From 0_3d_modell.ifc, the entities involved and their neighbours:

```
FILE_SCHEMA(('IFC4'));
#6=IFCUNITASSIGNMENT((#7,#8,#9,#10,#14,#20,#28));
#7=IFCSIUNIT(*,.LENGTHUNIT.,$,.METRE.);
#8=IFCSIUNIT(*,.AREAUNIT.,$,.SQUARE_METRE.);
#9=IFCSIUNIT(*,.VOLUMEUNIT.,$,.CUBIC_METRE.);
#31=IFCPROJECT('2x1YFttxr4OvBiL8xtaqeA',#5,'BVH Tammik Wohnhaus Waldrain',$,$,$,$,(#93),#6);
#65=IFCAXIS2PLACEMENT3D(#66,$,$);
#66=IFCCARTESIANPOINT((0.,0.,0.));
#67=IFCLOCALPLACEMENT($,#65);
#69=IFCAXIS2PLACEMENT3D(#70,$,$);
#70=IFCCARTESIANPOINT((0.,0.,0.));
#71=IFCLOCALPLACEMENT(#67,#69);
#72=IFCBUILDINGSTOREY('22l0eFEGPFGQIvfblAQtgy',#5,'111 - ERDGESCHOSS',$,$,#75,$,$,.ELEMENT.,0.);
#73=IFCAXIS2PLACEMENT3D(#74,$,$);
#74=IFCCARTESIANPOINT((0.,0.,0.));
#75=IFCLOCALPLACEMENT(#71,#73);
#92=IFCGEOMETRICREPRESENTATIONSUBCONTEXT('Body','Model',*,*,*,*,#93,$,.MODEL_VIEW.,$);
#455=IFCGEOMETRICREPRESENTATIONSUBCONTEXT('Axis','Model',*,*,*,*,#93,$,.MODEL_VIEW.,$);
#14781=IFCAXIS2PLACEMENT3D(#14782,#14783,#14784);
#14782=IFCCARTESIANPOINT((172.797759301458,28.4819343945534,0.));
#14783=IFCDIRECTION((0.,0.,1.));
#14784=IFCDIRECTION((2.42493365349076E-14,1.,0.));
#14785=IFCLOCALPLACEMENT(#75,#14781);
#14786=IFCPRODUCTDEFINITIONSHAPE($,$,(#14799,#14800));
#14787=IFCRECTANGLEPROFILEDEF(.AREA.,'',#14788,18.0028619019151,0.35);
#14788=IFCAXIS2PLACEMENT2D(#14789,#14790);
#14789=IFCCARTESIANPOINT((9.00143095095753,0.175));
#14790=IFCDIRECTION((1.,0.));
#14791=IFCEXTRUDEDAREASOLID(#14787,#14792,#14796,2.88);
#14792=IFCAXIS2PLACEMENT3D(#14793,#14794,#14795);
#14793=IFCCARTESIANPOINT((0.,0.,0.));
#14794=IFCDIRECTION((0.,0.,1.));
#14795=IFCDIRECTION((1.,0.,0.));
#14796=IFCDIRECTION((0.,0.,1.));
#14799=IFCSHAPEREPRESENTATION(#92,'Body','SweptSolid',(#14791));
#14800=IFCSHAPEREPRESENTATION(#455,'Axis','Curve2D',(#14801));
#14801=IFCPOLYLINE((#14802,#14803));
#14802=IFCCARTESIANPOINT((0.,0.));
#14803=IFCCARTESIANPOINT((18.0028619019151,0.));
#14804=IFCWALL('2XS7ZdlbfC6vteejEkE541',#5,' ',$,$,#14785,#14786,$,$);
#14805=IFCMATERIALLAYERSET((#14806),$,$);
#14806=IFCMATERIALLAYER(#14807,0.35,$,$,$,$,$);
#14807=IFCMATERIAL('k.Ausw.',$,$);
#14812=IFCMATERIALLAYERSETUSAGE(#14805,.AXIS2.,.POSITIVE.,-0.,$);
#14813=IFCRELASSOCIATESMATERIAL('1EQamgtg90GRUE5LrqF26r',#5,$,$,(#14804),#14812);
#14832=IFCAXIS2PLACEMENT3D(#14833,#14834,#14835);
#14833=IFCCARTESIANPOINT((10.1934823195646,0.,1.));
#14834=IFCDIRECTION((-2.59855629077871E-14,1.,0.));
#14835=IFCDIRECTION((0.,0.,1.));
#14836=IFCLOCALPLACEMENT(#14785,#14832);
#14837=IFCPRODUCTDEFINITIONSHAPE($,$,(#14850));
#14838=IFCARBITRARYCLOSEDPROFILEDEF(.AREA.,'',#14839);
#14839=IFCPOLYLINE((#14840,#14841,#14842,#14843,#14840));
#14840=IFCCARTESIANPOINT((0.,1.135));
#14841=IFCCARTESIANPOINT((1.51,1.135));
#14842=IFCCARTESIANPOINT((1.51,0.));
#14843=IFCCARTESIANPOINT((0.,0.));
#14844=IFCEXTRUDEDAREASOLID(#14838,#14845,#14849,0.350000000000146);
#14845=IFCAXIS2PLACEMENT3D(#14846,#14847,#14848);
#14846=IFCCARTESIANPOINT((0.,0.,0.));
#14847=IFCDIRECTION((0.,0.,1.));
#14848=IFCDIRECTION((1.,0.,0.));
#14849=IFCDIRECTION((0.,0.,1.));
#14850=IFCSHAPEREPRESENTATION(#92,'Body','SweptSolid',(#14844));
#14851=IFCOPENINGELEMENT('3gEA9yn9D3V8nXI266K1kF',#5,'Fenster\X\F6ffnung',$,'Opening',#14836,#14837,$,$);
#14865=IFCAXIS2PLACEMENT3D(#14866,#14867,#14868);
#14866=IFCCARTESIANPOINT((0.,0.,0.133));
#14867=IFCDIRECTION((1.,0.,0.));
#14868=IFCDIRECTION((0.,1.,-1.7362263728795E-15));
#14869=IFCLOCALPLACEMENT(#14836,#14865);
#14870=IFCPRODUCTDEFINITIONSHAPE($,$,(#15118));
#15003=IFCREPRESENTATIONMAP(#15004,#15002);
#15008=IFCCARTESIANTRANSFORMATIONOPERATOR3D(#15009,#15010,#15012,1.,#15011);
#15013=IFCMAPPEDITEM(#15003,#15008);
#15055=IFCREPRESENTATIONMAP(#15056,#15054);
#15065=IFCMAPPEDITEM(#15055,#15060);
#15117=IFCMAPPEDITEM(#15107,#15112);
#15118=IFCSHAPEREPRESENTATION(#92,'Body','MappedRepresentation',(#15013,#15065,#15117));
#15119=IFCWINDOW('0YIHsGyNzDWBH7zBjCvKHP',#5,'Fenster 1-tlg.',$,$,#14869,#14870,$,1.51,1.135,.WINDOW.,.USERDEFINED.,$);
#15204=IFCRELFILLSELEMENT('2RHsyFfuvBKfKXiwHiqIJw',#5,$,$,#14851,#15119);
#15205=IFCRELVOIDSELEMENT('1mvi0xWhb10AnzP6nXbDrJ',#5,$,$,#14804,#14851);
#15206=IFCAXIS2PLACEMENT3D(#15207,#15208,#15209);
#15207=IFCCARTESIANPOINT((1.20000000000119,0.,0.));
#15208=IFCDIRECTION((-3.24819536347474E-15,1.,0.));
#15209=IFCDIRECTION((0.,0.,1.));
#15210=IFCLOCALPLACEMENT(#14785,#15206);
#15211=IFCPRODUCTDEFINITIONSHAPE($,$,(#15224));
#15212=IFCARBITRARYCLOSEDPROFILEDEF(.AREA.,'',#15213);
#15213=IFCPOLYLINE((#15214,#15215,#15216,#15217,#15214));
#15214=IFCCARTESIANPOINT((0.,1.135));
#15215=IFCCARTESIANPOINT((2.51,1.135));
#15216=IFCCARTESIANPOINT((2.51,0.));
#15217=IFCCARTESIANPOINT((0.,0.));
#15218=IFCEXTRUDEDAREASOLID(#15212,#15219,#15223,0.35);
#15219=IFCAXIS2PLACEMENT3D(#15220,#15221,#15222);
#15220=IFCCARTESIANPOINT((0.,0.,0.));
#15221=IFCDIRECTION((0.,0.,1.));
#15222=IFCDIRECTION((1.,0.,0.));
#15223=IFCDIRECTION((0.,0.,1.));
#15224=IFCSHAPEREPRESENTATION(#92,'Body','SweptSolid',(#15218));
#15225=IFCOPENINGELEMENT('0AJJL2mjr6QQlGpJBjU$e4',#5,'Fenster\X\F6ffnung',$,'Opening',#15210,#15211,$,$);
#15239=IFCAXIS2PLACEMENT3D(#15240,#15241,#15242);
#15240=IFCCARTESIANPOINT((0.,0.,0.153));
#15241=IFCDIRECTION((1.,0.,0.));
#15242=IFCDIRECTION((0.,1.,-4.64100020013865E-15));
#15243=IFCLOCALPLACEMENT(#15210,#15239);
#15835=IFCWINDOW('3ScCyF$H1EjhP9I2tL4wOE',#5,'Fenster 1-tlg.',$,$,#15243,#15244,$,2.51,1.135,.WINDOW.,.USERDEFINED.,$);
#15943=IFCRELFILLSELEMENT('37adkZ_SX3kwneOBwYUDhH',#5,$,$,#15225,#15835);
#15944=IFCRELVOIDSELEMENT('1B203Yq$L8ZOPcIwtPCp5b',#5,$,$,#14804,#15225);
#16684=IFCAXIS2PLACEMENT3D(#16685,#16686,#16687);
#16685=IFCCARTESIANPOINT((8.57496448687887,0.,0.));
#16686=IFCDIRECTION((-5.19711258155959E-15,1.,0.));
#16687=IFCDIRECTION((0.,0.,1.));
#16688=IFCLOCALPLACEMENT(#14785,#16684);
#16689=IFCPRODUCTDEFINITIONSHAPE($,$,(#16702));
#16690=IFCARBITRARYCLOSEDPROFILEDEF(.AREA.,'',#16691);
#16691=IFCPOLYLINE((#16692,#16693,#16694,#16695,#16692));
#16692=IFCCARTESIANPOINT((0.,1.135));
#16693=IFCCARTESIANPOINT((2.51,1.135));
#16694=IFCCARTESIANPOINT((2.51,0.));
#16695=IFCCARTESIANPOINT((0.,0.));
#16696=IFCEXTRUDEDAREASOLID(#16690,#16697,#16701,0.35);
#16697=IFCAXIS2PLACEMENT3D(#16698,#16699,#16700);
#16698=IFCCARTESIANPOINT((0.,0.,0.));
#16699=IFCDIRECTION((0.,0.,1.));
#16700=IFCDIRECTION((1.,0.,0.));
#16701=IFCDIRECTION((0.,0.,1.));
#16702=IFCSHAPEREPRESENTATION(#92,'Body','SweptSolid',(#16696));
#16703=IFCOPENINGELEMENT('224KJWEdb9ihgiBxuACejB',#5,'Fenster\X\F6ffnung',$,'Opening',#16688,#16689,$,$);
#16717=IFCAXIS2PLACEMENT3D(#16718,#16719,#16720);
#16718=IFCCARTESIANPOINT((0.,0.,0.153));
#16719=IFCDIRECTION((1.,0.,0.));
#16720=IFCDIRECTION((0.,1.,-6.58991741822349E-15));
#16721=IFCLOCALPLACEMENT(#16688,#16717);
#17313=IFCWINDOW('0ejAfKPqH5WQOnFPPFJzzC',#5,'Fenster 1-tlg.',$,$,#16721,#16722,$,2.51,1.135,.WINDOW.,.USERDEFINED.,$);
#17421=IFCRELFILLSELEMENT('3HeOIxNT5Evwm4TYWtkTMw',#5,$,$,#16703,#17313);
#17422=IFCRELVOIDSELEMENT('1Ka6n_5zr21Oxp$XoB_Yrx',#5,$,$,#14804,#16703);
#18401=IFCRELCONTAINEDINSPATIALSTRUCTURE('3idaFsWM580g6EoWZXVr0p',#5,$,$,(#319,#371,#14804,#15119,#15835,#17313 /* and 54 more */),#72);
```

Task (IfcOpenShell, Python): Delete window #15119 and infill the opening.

```python
import ifcopenshell
import ifcopenshell.api.feature
import ifcopenshell.api.root
import ifcopenshell.geom
import ifcopenshell.util.shape

model = ifcopenshell.open("0_3d_modell.ifc")
settings = ifcopenshell.geom.settings()


def volume(element):
    """Net volume in cubic metres, openings subtracted."""
    shape = ifcopenshell.geom.create_shape(settings, element)
    return ifcopenshell.util.shape.get_volume(shape.geometry)


window = model.by_guid("0YIHsGyNzDWBH7zBjCvKHP")
opening = window.FillsVoids[0].RelatingOpeningElement
wall = opening.VoidsElements[0].RelatingBuildingElement
before = volume(wall)

ifcopenshell.api.root.remove_product(model, product=window)
ifcopenshell.api.feature.remove_feature(model, feature=opening)

after = volume(wall)

print(f"wall volume {before:.3f} -> {after:.3f} m3")

model.write("0_3d_modell-out.ifc")
```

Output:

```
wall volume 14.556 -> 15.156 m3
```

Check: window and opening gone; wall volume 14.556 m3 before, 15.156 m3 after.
